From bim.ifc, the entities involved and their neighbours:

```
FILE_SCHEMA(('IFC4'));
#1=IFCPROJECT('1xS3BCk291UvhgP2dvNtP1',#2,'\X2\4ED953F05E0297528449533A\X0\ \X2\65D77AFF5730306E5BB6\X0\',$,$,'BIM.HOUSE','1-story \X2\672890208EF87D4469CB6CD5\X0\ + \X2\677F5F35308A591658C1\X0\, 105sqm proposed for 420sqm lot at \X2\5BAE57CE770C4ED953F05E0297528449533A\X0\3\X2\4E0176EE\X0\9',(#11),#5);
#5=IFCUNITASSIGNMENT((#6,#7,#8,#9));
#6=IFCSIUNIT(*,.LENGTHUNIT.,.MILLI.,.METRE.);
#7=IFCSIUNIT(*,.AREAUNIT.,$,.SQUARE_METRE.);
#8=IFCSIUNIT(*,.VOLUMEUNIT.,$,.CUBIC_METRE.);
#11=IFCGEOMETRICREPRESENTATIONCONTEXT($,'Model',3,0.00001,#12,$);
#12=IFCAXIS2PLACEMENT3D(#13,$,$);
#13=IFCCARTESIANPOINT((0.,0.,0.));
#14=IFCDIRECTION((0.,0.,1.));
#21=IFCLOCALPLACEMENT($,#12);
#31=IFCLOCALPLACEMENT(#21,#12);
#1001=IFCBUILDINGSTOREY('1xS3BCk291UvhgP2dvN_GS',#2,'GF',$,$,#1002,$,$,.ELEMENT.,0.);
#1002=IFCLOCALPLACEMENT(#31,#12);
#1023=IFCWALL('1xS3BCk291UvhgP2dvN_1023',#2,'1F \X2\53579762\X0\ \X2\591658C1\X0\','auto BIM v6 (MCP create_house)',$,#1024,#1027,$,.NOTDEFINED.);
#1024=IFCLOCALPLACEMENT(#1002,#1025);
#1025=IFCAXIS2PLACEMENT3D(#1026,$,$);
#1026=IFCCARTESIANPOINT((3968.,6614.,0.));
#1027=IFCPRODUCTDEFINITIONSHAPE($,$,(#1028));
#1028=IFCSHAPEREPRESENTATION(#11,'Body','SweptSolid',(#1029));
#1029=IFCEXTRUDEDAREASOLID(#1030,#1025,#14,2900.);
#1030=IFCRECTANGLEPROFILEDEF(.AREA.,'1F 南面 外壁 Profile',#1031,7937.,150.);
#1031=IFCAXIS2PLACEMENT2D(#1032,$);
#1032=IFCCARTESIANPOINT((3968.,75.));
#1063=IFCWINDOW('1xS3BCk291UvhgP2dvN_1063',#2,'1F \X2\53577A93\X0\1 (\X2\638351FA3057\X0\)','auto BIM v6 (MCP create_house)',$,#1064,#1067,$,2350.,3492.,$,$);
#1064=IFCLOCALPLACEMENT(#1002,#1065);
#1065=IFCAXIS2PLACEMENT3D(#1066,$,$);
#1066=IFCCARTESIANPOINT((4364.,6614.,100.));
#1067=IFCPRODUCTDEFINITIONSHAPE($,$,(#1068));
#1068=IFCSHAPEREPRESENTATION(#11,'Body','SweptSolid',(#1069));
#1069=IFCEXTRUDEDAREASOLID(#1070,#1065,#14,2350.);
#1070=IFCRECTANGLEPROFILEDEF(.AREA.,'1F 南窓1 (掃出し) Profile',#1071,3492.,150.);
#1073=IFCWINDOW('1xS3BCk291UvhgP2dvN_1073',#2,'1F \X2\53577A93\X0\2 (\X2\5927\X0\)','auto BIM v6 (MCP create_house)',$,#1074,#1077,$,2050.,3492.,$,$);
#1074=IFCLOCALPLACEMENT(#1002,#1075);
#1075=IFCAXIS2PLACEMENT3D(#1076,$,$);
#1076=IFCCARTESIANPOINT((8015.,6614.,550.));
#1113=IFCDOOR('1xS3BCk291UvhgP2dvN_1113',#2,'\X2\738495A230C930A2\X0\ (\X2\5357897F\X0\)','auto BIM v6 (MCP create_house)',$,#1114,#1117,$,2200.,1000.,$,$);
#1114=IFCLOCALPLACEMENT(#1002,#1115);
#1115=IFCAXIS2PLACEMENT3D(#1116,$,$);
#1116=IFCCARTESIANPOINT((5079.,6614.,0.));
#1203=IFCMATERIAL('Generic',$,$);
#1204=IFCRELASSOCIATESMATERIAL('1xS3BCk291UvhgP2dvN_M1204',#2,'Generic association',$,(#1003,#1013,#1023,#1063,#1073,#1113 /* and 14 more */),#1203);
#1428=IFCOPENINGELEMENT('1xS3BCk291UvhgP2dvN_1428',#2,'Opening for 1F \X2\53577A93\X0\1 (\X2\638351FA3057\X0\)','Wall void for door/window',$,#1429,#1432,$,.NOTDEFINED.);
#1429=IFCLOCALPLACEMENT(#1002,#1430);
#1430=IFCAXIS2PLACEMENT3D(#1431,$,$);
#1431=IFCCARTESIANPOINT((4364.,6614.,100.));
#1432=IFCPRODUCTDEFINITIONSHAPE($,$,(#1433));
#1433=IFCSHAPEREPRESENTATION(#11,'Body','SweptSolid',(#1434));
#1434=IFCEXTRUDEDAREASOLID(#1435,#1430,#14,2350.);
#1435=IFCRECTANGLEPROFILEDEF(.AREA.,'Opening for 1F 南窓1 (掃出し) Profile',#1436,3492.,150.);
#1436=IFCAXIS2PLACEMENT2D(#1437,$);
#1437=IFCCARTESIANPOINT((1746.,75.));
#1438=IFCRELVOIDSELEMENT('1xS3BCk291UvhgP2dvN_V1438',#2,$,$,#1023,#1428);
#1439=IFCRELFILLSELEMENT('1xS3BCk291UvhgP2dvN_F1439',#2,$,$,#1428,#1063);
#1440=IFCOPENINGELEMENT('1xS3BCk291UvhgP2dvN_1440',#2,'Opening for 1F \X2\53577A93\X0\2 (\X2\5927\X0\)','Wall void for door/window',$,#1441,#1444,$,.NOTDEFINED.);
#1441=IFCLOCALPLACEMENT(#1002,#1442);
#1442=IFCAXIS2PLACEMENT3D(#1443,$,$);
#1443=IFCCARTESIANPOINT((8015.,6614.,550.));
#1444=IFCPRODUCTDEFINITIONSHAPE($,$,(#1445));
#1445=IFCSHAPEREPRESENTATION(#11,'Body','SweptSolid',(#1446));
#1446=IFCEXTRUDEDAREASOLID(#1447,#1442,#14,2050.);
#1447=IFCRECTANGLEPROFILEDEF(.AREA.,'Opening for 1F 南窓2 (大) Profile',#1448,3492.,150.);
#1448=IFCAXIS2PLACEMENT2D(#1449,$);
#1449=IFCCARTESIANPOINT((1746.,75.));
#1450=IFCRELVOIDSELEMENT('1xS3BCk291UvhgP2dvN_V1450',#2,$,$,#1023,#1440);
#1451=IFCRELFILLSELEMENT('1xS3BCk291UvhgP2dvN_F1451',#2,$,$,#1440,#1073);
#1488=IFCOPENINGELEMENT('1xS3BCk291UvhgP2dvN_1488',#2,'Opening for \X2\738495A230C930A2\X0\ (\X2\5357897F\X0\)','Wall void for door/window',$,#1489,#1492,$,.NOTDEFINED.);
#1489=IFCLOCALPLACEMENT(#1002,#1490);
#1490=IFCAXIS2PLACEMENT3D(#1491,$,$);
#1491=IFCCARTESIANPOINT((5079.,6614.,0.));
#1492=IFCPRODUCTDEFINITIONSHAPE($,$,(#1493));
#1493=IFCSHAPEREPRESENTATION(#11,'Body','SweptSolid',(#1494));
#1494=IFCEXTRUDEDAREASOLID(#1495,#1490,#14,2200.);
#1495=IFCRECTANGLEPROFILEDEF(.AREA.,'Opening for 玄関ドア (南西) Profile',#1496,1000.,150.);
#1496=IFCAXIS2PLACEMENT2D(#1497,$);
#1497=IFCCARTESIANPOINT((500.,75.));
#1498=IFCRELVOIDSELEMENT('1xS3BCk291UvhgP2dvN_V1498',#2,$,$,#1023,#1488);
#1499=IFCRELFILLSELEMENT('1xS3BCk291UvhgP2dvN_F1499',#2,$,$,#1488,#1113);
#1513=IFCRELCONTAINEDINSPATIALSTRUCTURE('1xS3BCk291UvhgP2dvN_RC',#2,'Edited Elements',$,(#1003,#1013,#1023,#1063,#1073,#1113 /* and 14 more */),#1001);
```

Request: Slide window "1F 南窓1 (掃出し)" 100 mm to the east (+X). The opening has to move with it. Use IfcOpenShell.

```python
import ifcopenshell
import ifcopenshell.api.geometry
import ifcopenshell.util.placement
import ifcopenshell.util.unit

model = ifcopenshell.open("bim.ifc")
unit_scale = ifcopenshell.util.unit.calculate_unit_scale(model)

window = model.by_guid("1xS3BCk291UvhgP2dvN_1063")
opening = window.FillsVoids[0].RelatingOpeningElement
wall = opening.VoidsElements[0].RelatingBuildingElement

wall_matrix = ifcopenshell.util.placement.get_local_placement(wall.ObjectPlacement)
shift = wall_matrix[:3, 0] * 0.1 / unit_scale
before = ifcopenshell.util.placement.get_local_placement(window.ObjectPlacement)[:3, 3].copy()

# The window is not placed relative to its opening, so move both.
for product in (opening, window):
    matrix = ifcopenshell.util.placement.get_local_placement(product.ObjectPlacement)
    matrix[:3, 3] += shift
    ifcopenshell.api.geometry.edit_object_placement(model, product=product, matrix=matrix, is_si=False)

after = ifcopenshell.util.placement.get_local_placement(window.ObjectPlacement)[:3, 3]
print("window moved by", (after - before).round(3) + 0.0)

model.write("bim-out.ifc")
```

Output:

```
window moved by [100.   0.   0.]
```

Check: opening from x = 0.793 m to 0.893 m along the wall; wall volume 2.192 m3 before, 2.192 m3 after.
